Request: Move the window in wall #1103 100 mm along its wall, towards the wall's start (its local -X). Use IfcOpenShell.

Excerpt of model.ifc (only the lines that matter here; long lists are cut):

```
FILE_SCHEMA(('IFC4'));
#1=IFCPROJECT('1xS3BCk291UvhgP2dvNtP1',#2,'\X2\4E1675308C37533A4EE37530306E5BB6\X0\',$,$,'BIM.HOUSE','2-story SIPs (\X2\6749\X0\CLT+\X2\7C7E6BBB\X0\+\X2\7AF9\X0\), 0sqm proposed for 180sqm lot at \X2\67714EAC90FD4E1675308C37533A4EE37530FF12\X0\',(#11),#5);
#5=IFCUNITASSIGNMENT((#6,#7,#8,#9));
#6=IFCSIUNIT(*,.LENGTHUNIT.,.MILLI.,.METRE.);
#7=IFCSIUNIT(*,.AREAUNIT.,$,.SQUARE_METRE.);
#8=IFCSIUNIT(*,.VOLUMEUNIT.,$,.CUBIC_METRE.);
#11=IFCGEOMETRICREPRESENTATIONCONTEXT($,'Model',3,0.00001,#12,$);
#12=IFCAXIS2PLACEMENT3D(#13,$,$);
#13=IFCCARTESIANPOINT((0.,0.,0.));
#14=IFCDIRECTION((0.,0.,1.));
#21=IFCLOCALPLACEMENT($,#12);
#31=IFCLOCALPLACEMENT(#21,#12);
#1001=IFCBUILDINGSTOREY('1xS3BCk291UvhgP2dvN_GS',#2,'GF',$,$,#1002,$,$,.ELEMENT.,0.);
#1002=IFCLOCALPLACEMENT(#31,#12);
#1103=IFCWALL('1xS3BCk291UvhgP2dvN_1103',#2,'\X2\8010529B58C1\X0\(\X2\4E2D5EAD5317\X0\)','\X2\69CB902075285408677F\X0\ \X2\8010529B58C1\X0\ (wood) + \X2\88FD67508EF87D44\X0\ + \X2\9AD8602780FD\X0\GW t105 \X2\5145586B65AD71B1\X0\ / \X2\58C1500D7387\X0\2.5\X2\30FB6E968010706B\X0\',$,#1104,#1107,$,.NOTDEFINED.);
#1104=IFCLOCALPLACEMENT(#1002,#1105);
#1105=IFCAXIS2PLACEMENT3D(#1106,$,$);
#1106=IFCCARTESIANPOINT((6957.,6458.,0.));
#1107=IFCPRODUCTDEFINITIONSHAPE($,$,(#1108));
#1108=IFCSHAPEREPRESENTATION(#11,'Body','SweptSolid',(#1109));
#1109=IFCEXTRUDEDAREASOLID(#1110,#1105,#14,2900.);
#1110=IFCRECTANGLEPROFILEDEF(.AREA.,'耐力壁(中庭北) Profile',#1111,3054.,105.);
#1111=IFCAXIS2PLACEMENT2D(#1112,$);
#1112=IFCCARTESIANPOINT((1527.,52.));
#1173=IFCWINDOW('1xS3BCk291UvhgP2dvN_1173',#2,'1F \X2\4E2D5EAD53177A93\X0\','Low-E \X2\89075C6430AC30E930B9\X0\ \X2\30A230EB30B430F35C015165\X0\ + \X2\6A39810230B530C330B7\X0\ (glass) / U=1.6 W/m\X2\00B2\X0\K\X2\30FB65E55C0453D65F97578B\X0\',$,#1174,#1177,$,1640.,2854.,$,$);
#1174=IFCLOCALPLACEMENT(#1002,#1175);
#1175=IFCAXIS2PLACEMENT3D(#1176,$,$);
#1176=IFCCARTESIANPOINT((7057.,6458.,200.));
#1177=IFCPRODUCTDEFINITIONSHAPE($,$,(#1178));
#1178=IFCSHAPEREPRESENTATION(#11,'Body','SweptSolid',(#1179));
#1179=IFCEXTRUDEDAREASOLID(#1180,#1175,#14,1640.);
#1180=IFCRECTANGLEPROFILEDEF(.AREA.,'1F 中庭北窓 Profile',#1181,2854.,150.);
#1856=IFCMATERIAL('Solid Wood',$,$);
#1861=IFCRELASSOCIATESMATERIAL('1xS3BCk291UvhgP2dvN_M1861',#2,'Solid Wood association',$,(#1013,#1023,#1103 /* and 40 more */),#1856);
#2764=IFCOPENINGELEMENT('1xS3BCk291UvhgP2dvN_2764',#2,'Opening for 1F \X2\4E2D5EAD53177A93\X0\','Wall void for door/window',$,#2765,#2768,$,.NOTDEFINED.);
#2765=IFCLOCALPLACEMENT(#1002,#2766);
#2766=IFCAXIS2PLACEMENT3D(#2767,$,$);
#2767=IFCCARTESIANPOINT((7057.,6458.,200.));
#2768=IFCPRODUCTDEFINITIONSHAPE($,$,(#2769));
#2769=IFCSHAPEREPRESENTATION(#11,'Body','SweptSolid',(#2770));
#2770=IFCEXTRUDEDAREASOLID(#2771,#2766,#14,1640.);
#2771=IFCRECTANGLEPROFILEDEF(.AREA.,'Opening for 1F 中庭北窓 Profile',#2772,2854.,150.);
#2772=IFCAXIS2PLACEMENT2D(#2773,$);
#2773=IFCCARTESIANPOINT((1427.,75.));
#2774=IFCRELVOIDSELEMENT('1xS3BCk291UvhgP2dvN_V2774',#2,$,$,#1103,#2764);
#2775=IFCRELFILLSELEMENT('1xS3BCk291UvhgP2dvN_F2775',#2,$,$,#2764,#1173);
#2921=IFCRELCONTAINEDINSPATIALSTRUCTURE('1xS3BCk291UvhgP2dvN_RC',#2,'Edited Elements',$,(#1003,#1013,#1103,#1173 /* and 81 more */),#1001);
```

```python
import ifcopenshell
import ifcopenshell.api.geometry
import ifcopenshell.util.placement
import ifcopenshell.util.unit

model = ifcopenshell.open("model.ifc")
unit_scale = ifcopenshell.util.unit.calculate_unit_scale(model)

window = model.by_id(1173)
opening = window.FillsVoids[0].RelatingOpeningElement
wall = opening.VoidsElements[0].RelatingBuildingElement

wall_matrix = ifcopenshell.util.placement.get_local_placement(wall.ObjectPlacement)
shift = wall_matrix[:3, 0] * -0.1 / unit_scale
before = ifcopenshell.util.placement.get_local_placement(window.ObjectPlacement)[:3, 3].copy()

# The window is not placed relative to its opening, so move both.
for product in (opening, window):
    matrix = ifcopenshell.util.placement.get_local_placement(product.ObjectPlacement)
    matrix[:3, 3] += shift
    ifcopenshell.api.geometry.edit_object_placement(model, product=product, matrix=matrix, is_si=False)

after = ifcopenshell.util.placement.get_local_placement(window.ObjectPlacement)[:3, 3]
print("window moved by", (after - before).round(3) + 0.0)

model.write("model_updated.ifc")
```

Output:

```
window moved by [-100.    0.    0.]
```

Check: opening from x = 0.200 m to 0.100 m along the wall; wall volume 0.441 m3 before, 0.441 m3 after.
